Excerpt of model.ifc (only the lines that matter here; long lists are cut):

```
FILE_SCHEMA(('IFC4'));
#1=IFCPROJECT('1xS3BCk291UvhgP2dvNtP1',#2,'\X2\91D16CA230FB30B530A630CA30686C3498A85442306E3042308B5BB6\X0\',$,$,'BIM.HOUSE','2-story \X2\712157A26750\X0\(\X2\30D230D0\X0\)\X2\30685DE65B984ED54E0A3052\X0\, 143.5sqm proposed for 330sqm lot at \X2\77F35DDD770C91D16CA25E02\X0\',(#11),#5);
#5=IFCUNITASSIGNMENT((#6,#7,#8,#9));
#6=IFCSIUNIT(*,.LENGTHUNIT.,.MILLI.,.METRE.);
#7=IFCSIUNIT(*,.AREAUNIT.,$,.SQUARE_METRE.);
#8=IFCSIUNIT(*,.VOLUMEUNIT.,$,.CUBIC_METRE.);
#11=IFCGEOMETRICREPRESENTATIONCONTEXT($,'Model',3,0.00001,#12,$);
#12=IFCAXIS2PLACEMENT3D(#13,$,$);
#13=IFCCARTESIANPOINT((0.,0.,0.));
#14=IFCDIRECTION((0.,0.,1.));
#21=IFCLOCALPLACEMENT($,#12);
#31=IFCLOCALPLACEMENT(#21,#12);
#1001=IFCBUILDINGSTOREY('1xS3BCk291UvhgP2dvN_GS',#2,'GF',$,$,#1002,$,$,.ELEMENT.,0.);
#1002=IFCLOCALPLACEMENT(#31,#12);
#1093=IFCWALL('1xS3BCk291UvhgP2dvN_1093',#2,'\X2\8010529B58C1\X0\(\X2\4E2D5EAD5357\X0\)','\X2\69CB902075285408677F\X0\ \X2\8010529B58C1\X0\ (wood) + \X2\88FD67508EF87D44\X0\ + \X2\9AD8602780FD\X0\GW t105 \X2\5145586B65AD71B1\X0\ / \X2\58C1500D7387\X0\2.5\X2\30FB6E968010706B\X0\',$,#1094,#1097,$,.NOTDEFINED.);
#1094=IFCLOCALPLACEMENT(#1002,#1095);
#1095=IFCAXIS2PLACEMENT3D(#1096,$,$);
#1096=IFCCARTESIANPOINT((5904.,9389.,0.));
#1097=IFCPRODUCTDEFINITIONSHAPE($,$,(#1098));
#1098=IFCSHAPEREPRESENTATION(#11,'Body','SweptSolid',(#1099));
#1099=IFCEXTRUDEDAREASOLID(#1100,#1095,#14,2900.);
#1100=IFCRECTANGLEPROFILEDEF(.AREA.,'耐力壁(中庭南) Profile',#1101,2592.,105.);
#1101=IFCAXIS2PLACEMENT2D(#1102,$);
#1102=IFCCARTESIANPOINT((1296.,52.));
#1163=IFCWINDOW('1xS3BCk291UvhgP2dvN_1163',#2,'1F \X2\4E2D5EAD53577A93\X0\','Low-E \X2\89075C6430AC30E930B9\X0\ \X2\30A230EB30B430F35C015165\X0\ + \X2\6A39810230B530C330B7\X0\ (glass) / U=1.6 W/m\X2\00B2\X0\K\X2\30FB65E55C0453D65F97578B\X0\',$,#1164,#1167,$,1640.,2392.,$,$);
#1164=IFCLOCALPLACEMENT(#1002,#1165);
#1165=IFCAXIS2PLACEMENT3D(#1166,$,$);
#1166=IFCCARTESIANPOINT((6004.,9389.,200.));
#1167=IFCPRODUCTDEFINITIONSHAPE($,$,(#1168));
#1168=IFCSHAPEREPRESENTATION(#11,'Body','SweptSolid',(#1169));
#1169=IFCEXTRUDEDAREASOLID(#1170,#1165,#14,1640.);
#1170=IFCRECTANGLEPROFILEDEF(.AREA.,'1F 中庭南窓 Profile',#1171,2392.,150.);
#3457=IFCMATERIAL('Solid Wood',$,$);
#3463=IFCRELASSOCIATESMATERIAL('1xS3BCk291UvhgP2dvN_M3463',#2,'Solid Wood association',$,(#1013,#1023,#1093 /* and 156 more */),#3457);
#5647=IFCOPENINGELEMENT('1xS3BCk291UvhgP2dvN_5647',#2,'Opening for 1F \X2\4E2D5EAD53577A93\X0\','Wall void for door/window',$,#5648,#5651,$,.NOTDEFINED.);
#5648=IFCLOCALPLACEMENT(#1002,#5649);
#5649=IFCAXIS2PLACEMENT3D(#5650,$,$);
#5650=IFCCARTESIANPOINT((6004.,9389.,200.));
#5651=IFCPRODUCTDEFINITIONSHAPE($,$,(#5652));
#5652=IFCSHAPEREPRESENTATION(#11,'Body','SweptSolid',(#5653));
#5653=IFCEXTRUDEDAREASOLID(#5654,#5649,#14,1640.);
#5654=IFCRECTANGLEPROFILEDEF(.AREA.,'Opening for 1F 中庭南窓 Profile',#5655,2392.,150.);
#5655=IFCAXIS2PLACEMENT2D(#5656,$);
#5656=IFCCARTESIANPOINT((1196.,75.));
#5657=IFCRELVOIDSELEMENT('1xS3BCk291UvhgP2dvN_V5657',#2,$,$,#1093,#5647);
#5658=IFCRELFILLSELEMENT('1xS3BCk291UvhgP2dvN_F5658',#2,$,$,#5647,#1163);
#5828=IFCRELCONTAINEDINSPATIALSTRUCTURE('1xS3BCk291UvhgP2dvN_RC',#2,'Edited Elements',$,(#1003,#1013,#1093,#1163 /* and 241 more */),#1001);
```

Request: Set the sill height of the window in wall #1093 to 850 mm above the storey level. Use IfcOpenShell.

```python
import numpy as np
import ifcopenshell
import ifcopenshell.api.geometry
import ifcopenshell.geom
import ifcopenshell.util.element
import ifcopenshell.util.placement
import ifcopenshell.util.shape
import ifcopenshell.util.unit

model = ifcopenshell.open("model.ifc")
unit_scale = ifcopenshell.util.unit.calculate_unit_scale(model)

window = model.by_guid("1xS3BCk291UvhgP2dvN_1163")
opening = window.FillsVoids[0].RelatingOpeningElement
storey = ifcopenshell.util.element.get_container(window, ifc_class="IfcBuildingStorey")
level = ifcopenshell.util.placement.get_local_placement(storey.ObjectPlacement)[2, 3]

# The opening's origin need not be at the sill, so measure its lowest point.
shape = ifcopenshell.geom.create_shape(ifcopenshell.geom.settings(), opening)
bottom = ifcopenshell.util.shape.get_shape_bottom_elevation(shape, shape.geometry) / unit_scale
dz = level + 0.85 / unit_scale - bottom

shift = np.array([0.0, 0.0, dz])
# The window is not placed relative to its opening, so move both.
for product in (opening, window):
    matrix = ifcopenshell.util.placement.get_local_placement(product.ObjectPlacement)
    matrix[:3, 3] += shift
    ifcopenshell.api.geometry.edit_object_placement(model, product=product, matrix=matrix, is_si=False)

print(f"moved by {dz * unit_scale:+.3f} m")

model.write("model_updated.ifc")
```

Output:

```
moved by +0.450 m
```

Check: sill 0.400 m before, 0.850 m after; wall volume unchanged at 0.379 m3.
